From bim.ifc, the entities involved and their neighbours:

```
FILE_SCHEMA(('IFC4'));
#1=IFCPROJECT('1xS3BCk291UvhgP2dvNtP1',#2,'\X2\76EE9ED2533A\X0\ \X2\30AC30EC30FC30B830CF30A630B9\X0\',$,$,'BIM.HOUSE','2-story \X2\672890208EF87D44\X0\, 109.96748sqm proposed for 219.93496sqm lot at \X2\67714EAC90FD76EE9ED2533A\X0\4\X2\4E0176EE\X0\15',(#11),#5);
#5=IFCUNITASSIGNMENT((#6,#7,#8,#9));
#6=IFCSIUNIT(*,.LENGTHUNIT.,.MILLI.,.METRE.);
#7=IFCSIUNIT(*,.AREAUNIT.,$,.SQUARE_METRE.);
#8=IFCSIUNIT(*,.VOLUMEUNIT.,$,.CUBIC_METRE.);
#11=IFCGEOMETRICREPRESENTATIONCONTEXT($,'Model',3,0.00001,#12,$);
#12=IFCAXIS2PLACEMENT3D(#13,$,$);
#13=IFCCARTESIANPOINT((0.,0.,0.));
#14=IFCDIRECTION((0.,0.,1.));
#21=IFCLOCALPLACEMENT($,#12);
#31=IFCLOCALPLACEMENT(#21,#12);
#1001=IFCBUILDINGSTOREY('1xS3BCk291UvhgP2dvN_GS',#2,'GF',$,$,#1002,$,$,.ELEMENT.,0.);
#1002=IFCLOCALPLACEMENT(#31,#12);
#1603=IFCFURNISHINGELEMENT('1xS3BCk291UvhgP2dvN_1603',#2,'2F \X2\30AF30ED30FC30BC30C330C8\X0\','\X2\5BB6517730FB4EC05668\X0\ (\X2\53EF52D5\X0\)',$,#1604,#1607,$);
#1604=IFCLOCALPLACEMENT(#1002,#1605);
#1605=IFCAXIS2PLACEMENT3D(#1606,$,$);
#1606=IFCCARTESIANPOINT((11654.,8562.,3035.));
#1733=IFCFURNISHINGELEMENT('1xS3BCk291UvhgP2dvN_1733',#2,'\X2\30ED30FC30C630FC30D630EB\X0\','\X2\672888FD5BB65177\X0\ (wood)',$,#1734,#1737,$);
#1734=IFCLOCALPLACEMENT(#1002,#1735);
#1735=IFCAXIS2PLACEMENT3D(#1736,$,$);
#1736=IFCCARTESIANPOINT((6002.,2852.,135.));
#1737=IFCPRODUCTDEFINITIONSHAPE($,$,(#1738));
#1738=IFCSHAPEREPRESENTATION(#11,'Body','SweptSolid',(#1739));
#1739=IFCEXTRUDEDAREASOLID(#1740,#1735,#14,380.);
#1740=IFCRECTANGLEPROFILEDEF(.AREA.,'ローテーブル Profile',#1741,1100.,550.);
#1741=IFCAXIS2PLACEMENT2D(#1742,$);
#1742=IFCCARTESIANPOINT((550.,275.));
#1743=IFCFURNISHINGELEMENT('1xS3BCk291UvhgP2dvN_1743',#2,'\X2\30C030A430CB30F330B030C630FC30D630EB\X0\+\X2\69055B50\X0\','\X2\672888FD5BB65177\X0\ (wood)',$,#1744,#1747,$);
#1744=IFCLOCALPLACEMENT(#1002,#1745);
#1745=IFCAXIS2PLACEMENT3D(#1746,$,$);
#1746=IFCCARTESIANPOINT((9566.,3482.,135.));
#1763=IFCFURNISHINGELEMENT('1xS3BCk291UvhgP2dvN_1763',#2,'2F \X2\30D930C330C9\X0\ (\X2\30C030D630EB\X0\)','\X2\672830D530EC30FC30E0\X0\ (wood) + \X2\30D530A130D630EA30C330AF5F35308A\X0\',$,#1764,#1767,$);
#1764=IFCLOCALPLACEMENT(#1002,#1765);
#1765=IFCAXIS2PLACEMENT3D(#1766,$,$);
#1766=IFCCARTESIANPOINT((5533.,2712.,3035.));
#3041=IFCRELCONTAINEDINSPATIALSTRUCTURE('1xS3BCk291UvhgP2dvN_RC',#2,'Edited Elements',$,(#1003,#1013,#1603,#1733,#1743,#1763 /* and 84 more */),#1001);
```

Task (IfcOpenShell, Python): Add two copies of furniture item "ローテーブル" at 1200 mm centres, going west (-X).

```python
import numpy as np
import ifcopenshell
import ifcopenshell.api.geometry
import ifcopenshell.api.root
import ifcopenshell.util.element
import ifcopenshell.util.placement
import ifcopenshell.util.unit

model = ifcopenshell.open("bim.ifc")
unit_scale = ifcopenshell.util.unit.calculate_unit_scale(model)


def reuse_history(source, copy):
    """copy_class also copies each property set's owner history, people and application; keep the originals."""
    for rel in copy.IsDefinedBy:
        if rel.is_a("IfcRelDefinesByProperties") and (history := rel.RelatingPropertyDefinition.OwnerHistory):
            rel.RelatingPropertyDefinition.OwnerHistory = source.OwnerHistory
            ifcopenshell.util.element.remove_deep2(model, history)


source = model.by_id(1733)
base = ifcopenshell.util.placement.get_local_placement(source.ObjectPlacement)
step = np.array([-1.0, 0.0, 0.0]) * 1.2 / unit_scale

for i in range(1, 3):
    copy = ifcopenshell.api.root.copy_class(model, product=source)
    copy.Representation = ifcopenshell.util.element.copy_deep(
        model, source.Representation, exclude=["IfcGeometricRepresentationContext", "IfcRepresentationMap"]
    )
    reuse_history(source, copy)
    matrix = base.copy()
    matrix[:3, 3] += i * step
    print("added at", matrix[:3, 3].round(3) + 0.0)
    ifcopenshell.api.geometry.edit_object_placement(model, product=copy, matrix=matrix, is_si=False)

model.write("bim_rev.ifc")
```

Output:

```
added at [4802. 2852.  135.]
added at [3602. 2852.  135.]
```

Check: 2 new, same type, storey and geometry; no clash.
